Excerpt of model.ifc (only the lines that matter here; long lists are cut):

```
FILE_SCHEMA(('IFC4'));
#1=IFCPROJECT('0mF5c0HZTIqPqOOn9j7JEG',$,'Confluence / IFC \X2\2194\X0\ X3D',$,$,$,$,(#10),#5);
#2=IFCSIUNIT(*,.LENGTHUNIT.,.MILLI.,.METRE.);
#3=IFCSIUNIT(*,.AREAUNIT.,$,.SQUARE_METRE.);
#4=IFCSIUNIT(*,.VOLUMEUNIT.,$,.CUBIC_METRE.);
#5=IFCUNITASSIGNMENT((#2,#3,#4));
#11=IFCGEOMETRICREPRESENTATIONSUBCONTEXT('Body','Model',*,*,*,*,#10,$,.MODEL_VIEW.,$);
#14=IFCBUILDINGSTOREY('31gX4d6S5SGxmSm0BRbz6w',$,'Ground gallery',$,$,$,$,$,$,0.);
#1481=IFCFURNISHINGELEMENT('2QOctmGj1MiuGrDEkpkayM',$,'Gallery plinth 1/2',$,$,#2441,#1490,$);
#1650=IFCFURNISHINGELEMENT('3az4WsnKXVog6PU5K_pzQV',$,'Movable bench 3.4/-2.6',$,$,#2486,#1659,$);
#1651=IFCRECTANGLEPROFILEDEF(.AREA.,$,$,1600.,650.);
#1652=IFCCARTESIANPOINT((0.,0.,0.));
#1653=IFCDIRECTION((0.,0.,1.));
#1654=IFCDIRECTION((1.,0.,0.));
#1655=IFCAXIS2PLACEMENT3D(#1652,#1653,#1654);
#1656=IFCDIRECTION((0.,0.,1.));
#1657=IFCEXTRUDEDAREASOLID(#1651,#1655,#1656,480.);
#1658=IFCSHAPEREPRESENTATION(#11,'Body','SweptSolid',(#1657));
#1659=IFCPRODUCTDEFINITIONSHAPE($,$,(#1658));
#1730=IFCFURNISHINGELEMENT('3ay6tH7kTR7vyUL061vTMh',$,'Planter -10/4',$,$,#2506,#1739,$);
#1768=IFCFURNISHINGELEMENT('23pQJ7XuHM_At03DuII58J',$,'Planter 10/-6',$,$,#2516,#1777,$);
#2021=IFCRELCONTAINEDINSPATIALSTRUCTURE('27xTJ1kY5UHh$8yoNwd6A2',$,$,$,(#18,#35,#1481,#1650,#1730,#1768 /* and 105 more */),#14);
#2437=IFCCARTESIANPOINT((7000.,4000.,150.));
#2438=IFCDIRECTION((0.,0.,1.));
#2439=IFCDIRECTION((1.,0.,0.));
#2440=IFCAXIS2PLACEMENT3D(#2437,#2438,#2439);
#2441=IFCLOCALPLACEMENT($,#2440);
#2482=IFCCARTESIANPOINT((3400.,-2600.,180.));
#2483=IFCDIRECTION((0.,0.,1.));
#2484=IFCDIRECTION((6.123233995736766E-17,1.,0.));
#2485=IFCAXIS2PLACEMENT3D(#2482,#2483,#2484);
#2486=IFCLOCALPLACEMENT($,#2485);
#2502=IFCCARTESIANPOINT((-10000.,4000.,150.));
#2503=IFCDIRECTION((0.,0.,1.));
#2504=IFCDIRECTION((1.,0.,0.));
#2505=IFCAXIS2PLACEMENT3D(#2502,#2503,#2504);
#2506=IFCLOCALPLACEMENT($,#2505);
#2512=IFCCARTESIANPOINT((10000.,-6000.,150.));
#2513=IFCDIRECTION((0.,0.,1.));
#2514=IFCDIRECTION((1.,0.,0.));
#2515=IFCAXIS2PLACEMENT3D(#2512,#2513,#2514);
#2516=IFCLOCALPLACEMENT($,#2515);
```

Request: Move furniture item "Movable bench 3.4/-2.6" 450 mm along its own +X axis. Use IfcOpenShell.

```python
import ifcopenshell
import ifcopenshell.api.geometry
import ifcopenshell.util.placement
import ifcopenshell.util.unit

model = ifcopenshell.open("model.ifc")
unit_scale = ifcopenshell.util.unit.calculate_unit_scale(model)

item = model.by_guid("3az4WsnKXVog6PU5K_pzQV")
matrix = ifcopenshell.util.placement.get_local_placement(item.ObjectPlacement)
matrix[:3, 3] += matrix[:3, 0] * 0.45 / unit_scale
ifcopenshell.api.geometry.edit_object_placement(model, product=item, matrix=matrix, is_si=False)

print(ifcopenshell.util.placement.get_local_placement(item.ObjectPlacement).round(3) + 0.0)

model.write("model_updated.ifc")
```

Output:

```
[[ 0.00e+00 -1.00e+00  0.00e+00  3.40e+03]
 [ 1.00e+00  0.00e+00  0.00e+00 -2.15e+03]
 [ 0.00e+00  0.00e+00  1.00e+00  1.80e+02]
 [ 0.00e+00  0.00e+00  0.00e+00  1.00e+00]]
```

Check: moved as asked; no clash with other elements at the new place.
